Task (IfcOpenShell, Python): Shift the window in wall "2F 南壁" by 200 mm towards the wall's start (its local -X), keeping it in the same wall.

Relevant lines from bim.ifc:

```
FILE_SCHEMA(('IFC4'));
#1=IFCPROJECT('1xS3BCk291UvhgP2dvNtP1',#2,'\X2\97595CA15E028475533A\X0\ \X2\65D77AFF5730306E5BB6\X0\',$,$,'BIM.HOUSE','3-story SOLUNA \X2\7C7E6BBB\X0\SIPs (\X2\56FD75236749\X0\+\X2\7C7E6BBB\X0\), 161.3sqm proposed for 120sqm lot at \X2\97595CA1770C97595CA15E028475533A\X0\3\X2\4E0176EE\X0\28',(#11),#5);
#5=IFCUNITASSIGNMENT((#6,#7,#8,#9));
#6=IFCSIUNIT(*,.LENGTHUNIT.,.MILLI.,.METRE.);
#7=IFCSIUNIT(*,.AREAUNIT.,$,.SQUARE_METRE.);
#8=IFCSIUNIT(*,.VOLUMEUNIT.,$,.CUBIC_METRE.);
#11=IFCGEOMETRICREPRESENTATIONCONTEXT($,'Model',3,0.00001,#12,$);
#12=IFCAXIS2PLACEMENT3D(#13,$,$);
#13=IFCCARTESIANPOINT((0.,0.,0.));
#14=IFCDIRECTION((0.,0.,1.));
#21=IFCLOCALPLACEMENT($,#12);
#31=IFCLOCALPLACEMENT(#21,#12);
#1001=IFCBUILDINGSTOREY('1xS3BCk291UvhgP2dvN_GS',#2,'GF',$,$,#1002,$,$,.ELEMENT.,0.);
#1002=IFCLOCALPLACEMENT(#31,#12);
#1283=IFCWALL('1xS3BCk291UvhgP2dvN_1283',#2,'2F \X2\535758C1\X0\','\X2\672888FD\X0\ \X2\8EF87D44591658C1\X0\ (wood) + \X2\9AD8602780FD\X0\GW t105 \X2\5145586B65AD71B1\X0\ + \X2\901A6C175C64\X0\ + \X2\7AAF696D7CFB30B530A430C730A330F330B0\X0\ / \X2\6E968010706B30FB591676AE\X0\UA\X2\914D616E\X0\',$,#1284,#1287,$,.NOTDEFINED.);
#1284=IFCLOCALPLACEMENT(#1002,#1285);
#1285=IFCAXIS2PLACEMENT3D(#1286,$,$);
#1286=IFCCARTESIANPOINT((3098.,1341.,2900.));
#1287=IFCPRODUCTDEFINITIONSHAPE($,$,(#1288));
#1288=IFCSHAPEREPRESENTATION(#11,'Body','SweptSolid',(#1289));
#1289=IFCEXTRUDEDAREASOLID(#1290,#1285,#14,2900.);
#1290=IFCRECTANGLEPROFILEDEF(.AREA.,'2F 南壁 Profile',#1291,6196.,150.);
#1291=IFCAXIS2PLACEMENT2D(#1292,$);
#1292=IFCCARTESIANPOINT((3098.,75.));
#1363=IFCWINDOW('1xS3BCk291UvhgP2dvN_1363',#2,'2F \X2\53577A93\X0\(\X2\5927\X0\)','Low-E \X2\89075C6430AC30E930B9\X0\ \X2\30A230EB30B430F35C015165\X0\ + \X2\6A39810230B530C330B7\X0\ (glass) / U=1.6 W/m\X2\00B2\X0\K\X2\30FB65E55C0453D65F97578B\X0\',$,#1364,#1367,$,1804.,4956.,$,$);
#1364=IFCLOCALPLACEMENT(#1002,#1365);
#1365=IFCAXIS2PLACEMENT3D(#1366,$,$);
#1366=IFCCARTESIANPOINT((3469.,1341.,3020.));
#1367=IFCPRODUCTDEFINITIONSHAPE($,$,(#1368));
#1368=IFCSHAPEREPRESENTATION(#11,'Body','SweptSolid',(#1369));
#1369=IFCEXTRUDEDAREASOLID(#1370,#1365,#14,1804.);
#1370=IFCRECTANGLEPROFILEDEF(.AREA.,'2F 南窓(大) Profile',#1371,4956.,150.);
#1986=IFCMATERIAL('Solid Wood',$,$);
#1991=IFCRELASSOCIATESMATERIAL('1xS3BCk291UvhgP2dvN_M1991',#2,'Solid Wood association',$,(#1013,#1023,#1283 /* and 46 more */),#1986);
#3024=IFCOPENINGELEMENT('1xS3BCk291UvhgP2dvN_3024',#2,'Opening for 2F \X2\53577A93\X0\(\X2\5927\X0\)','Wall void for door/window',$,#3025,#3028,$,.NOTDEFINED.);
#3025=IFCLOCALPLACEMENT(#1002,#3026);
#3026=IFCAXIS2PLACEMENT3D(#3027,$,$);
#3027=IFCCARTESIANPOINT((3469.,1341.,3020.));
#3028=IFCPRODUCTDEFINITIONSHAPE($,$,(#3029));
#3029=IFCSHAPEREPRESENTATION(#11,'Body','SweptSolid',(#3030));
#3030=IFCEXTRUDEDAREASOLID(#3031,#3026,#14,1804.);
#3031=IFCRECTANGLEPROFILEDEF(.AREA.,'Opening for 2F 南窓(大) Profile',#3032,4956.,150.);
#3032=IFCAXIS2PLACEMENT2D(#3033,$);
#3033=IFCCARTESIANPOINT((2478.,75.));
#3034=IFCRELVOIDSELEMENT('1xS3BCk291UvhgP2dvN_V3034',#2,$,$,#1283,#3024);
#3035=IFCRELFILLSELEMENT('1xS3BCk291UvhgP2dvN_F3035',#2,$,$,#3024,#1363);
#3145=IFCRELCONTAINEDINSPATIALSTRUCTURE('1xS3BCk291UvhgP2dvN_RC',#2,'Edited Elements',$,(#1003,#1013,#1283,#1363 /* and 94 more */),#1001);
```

```python
import ifcopenshell
import ifcopenshell.api.geometry
import ifcopenshell.util.placement

model = ifcopenshell.open("bim.ifc")

window = model.by_id(1363)
opening = window.FillsVoids[0].RelatingOpeningElement
wall = opening.VoidsElements[0].RelatingBuildingElement

wall_matrix = ifcopenshell.util.placement.get_local_placement(wall.ObjectPlacement)
shift = wall_matrix[:3, 0] * -200.0
before = ifcopenshell.util.placement.get_local_placement(window.ObjectPlacement)[:3, 3].copy()

# The window is not placed relative to its opening, so move both.
for product in (opening, window):
    matrix = ifcopenshell.util.placement.get_local_placement(product.ObjectPlacement)
    matrix[:3, 3] += shift
    ifcopenshell.api.geometry.edit_object_placement(model, product=product, matrix=matrix, is_si=False)

after = ifcopenshell.util.placement.get_local_placement(window.ObjectPlacement)[:3, 3]
print("window moved by", (after - before).round(3) + 0.0)

model.write("bim_v2.ifc")
```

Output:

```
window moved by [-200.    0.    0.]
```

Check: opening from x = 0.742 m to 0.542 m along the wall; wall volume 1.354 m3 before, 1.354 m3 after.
